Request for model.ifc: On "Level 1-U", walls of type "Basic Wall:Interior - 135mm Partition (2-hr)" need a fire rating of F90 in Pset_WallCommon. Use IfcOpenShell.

First a look at what the model holds.

```python
import ifcopenshell
import ifcopenshell.util.element

model = ifcopenshell.open("model.ifc")
print(model.schema)
storey = next(s for s in model.by_type("IfcBuildingStorey") if s.Name == "Level 1-U")
walls = [e for e in ifcopenshell.util.element.get_decomposition(storey) if e.is_a("IfcWall")]
seen = {}
for e in walls:
    element_type = ifcopenshell.util.element.get_type(e)
    key = (element_type.Name if element_type != e and element_type else None, ifcopenshell.util.element.get_pset(e, "Pset_WallCommon", "FireRating"))
    seen[key] = seen.get(key, 0) + 1
for (name, value), count in sorted(seen.items(), key=str):
    print(count, "x", name, "|", value)
```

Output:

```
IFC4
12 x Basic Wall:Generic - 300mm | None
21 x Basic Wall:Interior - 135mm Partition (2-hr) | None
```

```python
import ifcopenshell
import ifcopenshell.api.pset
import ifcopenshell.util.element

model = ifcopenshell.open("model.ifc")

storey = next(s for s in model.by_type("IfcBuildingStorey") if s.Name == "Level 1-U")
walls = [e for e in ifcopenshell.util.element.get_decomposition(storey) if e.is_a("IfcWall")]

count = 0
for e in walls:
    element_type = ifcopenshell.util.element.get_type(e)
    if element_type in (None, e) or element_type.Name != "Basic Wall:Interior - 135mm Partition (2-hr)":
        continue
    # add_pset returns the element's existing set when there is one.
    pset = ifcopenshell.api.pset.add_pset(model, product=e, name="Pset_WallCommon")
    ifcopenshell.api.pset.edit_pset(model, pset=pset, properties={"FireRating": "F90"})
    count += 1

print(count, "walls updated")

model.write("model-out.ifc")
```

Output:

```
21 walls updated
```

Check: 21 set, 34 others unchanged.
